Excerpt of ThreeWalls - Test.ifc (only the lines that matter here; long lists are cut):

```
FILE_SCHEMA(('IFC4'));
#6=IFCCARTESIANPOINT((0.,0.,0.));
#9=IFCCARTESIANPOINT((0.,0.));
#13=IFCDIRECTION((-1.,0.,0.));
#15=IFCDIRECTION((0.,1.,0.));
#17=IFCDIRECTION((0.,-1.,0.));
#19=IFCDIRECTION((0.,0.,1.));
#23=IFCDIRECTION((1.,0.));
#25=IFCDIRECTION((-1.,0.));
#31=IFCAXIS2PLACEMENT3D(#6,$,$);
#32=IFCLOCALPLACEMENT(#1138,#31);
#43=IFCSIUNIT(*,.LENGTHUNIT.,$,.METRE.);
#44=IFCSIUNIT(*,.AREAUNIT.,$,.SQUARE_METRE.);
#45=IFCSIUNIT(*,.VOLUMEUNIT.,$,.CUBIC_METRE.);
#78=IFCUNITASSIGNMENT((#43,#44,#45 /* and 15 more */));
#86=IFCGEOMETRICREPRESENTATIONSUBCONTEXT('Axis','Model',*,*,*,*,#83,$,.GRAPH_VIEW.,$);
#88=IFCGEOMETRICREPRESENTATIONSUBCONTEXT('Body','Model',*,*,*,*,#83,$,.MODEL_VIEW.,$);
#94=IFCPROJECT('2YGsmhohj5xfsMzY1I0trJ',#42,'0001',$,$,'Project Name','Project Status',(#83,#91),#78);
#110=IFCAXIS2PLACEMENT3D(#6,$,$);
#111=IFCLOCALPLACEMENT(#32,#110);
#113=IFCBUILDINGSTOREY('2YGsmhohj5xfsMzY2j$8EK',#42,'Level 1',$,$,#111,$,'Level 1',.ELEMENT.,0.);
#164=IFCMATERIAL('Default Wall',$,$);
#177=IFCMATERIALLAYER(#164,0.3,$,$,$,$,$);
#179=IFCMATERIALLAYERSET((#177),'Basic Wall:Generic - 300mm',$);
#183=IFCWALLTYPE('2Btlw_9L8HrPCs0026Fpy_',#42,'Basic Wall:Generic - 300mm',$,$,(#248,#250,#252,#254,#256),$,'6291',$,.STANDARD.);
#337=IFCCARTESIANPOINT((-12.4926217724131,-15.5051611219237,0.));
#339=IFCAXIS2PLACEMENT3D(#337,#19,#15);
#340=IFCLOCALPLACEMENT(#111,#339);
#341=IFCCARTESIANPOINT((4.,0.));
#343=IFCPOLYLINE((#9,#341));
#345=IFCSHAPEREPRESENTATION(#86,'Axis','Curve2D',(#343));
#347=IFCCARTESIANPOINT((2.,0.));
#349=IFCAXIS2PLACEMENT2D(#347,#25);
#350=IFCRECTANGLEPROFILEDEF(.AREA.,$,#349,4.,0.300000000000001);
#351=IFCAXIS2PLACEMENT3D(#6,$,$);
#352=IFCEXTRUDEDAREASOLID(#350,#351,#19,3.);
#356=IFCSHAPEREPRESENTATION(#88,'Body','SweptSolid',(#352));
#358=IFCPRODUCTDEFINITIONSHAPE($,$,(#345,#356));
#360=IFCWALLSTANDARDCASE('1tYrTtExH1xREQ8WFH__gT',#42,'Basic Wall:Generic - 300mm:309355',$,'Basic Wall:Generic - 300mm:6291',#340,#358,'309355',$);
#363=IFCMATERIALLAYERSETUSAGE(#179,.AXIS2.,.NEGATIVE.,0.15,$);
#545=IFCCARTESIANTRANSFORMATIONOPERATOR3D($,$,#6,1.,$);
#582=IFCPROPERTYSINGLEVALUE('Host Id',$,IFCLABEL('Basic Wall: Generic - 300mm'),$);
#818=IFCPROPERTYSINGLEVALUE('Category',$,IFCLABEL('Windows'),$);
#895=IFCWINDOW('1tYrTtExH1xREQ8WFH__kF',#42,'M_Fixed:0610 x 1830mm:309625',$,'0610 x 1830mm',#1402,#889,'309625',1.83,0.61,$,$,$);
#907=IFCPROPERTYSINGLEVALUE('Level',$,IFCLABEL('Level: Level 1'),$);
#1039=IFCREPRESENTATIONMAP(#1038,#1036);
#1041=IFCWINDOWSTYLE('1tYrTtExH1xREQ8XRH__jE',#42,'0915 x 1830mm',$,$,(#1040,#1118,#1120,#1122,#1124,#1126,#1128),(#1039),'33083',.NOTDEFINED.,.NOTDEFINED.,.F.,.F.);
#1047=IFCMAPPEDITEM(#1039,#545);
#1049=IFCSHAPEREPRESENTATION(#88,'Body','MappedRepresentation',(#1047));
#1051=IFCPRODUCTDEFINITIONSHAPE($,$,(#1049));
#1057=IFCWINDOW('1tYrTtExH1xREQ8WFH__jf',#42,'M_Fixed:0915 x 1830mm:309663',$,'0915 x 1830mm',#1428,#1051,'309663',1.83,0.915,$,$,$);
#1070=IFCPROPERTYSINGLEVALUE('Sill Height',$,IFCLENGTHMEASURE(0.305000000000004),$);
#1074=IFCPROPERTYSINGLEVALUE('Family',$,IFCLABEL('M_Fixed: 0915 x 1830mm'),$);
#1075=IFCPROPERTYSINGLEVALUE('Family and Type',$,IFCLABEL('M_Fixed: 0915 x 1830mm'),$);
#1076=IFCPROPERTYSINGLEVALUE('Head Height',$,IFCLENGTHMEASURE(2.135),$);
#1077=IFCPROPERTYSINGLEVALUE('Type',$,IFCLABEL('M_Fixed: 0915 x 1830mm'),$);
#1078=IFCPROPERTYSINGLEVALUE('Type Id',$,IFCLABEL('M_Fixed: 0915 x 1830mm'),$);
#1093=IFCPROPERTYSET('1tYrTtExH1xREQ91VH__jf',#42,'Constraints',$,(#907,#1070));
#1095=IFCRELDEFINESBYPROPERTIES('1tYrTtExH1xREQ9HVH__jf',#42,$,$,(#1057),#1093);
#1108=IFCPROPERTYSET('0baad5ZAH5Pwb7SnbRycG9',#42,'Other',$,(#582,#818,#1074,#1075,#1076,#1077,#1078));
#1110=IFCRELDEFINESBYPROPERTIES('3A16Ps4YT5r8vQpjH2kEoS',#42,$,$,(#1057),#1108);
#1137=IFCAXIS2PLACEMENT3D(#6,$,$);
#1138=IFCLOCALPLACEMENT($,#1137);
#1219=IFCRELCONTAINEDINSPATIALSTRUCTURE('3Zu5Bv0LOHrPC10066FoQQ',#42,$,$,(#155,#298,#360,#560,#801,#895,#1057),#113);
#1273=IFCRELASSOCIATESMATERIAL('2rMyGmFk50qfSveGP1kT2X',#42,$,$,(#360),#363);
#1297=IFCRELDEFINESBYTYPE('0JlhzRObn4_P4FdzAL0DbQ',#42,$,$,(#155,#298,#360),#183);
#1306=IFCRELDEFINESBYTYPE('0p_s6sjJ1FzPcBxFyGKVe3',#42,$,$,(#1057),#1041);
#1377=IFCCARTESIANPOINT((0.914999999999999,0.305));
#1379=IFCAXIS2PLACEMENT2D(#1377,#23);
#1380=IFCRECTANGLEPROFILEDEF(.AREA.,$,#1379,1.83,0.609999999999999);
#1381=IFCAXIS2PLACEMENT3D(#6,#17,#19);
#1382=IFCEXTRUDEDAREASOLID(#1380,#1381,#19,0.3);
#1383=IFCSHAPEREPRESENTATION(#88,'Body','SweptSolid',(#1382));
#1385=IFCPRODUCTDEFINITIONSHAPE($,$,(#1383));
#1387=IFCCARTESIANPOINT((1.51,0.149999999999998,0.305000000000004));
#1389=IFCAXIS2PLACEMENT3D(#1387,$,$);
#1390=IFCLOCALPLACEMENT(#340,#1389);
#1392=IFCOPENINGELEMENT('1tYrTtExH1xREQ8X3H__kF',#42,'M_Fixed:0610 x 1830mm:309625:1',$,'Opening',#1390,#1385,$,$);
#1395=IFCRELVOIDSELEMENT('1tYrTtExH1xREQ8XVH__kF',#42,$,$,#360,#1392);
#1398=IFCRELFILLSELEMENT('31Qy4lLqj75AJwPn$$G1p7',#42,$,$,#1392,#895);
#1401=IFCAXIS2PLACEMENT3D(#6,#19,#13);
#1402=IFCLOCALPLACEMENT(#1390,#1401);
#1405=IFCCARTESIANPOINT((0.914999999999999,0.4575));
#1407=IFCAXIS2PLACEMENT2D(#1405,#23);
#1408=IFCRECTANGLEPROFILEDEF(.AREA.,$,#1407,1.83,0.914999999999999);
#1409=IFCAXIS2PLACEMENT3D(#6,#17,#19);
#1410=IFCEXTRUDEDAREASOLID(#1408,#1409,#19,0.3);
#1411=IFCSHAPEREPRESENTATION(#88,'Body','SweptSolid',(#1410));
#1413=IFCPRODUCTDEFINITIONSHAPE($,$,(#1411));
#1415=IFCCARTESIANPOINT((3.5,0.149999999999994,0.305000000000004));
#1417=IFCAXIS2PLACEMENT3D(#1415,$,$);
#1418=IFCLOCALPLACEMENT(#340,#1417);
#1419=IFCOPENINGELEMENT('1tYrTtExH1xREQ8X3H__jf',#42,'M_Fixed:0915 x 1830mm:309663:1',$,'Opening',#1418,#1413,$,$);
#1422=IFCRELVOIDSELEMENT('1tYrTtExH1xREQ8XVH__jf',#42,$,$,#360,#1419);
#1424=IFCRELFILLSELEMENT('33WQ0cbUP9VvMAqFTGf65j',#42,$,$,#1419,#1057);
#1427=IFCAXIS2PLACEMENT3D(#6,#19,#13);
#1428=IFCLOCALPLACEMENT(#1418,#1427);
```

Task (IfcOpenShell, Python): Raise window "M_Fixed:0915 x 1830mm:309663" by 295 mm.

```python
import numpy as np
import ifcopenshell
import ifcopenshell.api.geometry
import ifcopenshell.api.pset
import ifcopenshell.util.element
import ifcopenshell.util.placement
import ifcopenshell.util.unit

model = ifcopenshell.open("ThreeWalls - Test.ifc")
unit_scale = ifcopenshell.util.unit.calculate_unit_scale(model)

window = model.by_id(1057)
opening = window.FillsVoids[0].RelatingOpeningElement
dz = 0.295 / unit_scale

shift = np.array([0.0, 0.0, dz])
# The window is placed relative to its opening, so it follows when the opening moves.
matrix = ifcopenshell.util.placement.get_local_placement(opening.ObjectPlacement)
matrix[:3, 3] += shift
ifcopenshell.api.geometry.edit_object_placement(
    model, product=opening, matrix=matrix, is_si=False, should_transform_children=True
)

# Keep the stored heights in step.
pset = model.by_id(ifcopenshell.util.element.get_pset(window, "Constraints", should_inherit=False)["id"])
ifcopenshell.api.pset.edit_pset(model, pset=pset, properties={
    "Sill Height": model.create_entity("IfcLengthMeasure", ifcopenshell.util.element.get_pset(window, "Constraints", "Sill Height") + dz),
})
pset = model.by_id(ifcopenshell.util.element.get_pset(window, "Other", should_inherit=False)["id"])
ifcopenshell.api.pset.edit_pset(model, pset=pset, properties={
    "Head Height": model.create_entity("IfcLengthMeasure", ifcopenshell.util.element.get_pset(window, "Other", "Head Height") + dz),
})

print(f"moved by {dz * unit_scale:+.3f} m")

model.write("ThreeWalls - Test_rev.ifc")
```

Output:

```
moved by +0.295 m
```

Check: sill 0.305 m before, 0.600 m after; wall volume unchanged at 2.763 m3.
